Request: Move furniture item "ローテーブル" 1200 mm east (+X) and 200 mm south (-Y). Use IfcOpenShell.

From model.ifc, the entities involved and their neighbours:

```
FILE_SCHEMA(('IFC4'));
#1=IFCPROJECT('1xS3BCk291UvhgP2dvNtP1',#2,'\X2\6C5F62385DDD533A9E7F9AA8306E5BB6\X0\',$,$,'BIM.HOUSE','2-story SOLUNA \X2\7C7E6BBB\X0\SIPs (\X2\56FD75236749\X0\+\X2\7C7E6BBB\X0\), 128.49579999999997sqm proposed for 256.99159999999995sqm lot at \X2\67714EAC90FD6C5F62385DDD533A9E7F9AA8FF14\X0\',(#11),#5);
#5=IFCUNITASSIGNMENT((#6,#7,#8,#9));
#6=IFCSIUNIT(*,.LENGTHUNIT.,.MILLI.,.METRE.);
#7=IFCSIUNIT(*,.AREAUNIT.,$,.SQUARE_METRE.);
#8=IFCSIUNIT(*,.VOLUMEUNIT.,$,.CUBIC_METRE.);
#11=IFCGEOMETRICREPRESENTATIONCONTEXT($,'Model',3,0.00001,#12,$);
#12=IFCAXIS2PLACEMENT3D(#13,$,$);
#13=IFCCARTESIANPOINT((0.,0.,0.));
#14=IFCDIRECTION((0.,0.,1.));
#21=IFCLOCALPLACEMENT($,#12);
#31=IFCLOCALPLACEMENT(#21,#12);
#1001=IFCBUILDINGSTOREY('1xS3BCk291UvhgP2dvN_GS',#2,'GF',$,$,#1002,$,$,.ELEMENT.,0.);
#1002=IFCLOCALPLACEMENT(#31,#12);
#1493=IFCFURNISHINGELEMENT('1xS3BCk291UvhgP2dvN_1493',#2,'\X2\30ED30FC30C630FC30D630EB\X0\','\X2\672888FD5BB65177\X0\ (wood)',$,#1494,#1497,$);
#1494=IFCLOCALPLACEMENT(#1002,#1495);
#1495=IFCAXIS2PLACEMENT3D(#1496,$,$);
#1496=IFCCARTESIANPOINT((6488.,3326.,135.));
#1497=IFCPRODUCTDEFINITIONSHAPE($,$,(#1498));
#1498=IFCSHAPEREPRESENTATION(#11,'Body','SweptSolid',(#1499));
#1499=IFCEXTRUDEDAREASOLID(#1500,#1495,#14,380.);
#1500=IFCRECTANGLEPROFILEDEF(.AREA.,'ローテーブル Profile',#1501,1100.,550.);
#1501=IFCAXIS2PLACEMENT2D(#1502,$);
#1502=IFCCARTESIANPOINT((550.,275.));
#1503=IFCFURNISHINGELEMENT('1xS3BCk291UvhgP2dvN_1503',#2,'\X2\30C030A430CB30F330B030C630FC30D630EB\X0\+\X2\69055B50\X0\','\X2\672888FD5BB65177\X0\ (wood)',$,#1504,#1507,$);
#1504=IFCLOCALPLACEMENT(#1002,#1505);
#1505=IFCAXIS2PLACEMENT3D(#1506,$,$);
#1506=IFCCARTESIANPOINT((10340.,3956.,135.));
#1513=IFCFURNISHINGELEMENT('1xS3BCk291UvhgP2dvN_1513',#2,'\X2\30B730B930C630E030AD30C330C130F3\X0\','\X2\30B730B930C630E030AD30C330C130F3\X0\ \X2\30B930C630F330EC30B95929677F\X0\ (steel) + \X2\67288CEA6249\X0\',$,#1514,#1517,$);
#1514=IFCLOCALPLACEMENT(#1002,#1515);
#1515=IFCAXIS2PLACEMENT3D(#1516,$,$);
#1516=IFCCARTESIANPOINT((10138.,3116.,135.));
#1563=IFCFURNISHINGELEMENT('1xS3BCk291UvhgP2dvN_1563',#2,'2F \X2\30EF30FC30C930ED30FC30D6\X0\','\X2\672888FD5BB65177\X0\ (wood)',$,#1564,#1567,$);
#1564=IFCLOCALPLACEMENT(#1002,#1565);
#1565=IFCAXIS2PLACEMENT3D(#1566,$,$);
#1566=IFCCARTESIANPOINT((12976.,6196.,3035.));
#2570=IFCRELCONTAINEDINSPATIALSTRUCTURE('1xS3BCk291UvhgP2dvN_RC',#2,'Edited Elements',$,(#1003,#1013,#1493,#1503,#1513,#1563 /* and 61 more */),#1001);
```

```python
import ifcopenshell
import ifcopenshell.api.geometry
import ifcopenshell.util.placement

model = ifcopenshell.open("model.ifc")

item = model.by_guid("1xS3BCk291UvhgP2dvN_1493")
matrix = ifcopenshell.util.placement.get_local_placement(item.ObjectPlacement)
matrix[0, 3] += 1200.0
matrix[1, 3] -= 200.0
ifcopenshell.api.geometry.edit_object_placement(model, product=item, matrix=matrix, is_si=False)

print(ifcopenshell.util.placement.get_local_placement(item.ObjectPlacement).round(3) + 0.0)

model.write("model_rev.ifc")
```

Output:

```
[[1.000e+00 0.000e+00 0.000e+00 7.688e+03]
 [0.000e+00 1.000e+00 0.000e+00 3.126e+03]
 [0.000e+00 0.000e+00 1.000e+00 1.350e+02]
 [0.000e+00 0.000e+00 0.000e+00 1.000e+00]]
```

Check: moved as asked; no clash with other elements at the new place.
